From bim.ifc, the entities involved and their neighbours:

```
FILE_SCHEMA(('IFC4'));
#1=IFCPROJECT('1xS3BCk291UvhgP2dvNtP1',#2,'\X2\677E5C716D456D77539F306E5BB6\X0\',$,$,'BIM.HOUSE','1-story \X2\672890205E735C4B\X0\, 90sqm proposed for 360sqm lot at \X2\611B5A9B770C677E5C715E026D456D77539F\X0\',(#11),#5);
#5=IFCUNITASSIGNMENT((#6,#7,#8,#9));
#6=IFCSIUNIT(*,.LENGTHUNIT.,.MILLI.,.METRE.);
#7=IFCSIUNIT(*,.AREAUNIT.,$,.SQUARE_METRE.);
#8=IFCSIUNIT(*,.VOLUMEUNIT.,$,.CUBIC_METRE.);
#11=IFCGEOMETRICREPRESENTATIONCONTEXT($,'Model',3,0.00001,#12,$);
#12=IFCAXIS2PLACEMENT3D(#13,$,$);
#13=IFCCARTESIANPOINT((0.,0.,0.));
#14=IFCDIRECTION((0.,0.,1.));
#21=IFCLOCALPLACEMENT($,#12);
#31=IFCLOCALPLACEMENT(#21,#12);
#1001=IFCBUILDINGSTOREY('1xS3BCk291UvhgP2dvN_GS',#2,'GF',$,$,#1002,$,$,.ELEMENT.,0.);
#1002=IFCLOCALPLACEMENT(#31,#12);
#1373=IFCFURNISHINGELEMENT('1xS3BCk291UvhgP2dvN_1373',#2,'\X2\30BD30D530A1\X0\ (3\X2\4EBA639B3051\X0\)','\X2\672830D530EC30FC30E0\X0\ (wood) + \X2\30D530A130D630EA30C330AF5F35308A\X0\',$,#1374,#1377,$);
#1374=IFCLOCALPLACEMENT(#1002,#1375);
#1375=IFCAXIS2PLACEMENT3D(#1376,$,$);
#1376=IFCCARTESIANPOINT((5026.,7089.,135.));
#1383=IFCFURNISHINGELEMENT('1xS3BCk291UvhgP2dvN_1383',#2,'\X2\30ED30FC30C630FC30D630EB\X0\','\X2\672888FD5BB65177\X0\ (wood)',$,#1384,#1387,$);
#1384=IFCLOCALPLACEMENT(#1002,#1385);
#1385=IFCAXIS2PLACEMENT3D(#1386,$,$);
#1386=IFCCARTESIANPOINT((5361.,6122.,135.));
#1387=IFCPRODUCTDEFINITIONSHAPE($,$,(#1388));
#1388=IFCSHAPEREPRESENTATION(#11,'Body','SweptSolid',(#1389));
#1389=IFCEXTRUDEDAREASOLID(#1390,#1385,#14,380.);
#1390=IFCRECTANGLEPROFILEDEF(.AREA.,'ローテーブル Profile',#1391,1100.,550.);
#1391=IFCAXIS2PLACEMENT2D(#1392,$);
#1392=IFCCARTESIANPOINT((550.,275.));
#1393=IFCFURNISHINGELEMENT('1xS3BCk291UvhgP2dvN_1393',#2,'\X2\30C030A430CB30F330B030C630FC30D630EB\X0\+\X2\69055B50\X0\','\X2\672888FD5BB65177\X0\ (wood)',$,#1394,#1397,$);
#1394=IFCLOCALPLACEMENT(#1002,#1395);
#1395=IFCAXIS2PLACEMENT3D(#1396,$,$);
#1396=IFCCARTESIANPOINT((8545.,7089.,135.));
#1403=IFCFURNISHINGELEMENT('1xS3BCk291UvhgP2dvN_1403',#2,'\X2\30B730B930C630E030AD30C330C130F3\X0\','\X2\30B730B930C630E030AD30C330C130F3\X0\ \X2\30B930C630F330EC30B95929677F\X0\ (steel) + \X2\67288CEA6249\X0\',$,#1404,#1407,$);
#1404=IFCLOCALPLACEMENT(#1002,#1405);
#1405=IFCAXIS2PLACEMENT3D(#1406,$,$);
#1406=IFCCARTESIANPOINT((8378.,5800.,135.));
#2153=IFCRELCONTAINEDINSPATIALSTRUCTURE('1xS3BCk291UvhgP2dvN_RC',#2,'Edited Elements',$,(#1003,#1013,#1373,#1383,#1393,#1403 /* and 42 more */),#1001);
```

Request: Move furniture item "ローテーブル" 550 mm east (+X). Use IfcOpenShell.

```python
import ifcopenshell
import ifcopenshell.api.geometry
import ifcopenshell.util.placement

model = ifcopenshell.open("bim.ifc")

item = model.by_guid("1xS3BCk291UvhgP2dvN_1383")
matrix = ifcopenshell.util.placement.get_local_placement(item.ObjectPlacement)
matrix[0, 3] += 550.0
ifcopenshell.api.geometry.edit_object_placement(model, product=item, matrix=matrix, is_si=False)

print(ifcopenshell.util.placement.get_local_placement(item.ObjectPlacement).round(3) + 0.0)

model.write("bim-out.ifc")
```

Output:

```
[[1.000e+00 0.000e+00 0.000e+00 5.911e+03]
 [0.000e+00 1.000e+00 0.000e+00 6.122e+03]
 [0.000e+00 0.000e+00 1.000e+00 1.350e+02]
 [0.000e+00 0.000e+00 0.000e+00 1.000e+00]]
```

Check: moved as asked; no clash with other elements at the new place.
